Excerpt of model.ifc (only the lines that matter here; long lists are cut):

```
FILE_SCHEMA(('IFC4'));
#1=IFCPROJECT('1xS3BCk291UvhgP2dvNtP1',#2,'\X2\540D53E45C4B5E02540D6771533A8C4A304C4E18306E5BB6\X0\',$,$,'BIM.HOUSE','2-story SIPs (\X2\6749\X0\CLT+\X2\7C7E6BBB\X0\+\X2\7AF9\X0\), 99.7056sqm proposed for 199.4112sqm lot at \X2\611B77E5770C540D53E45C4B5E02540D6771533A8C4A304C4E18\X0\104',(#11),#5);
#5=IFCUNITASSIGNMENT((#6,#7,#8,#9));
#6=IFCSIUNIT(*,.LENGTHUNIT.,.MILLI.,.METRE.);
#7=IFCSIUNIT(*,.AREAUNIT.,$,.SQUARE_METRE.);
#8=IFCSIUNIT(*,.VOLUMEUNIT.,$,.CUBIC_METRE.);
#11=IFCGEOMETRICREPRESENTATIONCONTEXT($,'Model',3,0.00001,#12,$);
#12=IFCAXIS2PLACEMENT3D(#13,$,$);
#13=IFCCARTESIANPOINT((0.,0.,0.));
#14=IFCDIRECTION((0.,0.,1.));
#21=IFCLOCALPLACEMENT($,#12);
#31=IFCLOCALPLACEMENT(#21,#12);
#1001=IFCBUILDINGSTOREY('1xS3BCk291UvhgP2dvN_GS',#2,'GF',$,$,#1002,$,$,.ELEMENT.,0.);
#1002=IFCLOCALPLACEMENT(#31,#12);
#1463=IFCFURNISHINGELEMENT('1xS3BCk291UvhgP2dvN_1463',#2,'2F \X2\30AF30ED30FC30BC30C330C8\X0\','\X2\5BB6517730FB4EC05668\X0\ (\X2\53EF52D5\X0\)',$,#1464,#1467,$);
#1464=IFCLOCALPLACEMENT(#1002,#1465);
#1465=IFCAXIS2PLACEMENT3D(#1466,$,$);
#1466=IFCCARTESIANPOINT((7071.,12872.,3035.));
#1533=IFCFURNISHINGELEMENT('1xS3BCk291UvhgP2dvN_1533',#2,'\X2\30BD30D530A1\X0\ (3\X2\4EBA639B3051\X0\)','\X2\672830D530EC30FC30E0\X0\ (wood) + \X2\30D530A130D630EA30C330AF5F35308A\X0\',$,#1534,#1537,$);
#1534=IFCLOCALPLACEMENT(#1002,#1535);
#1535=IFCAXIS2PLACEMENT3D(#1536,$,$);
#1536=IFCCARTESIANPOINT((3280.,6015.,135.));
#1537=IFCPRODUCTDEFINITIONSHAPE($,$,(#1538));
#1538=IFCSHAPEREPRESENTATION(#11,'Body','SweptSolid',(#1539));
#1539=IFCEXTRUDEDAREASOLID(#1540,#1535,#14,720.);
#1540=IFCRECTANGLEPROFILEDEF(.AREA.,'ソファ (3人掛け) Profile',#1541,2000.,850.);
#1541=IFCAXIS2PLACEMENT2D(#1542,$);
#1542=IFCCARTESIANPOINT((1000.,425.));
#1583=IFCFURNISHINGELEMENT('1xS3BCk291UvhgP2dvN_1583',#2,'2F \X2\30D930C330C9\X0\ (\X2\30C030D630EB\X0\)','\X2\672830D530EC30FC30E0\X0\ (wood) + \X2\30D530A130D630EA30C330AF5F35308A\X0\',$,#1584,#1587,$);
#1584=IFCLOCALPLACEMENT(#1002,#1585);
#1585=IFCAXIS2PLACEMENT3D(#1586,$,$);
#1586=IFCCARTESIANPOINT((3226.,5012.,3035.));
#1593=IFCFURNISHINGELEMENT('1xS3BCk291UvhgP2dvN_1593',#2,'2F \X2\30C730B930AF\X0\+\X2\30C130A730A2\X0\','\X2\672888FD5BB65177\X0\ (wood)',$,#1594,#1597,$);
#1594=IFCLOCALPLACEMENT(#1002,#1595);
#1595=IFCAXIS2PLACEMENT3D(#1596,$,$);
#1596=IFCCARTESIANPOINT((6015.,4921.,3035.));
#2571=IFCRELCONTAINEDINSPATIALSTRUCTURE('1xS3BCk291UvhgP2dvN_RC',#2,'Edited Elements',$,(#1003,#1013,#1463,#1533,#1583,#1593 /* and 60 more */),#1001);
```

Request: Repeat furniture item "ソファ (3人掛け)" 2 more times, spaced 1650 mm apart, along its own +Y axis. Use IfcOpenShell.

```python
import ifcopenshell
import ifcopenshell.api.geometry
import ifcopenshell.api.root
import ifcopenshell.util.element
import ifcopenshell.util.placement
import ifcopenshell.util.unit

model = ifcopenshell.open("model.ifc")
unit_scale = ifcopenshell.util.unit.calculate_unit_scale(model)


def reuse_history(source, copy):
    """copy_class also copies each property set's owner history, people and application; keep the originals."""
    for rel in copy.IsDefinedBy:
        if rel.is_a("IfcRelDefinesByProperties") and (history := rel.RelatingPropertyDefinition.OwnerHistory):
            rel.RelatingPropertyDefinition.OwnerHistory = source.OwnerHistory
            ifcopenshell.util.element.remove_deep2(model, history)


source = model.by_guid("1xS3BCk291UvhgP2dvN_1533")
base = ifcopenshell.util.placement.get_local_placement(source.ObjectPlacement)
step = base[:3, 1] * 1.65 / unit_scale

for i in range(1, 3):
    copy = ifcopenshell.api.root.copy_class(model, product=source)
    copy.Representation = ifcopenshell.util.element.copy_deep(
        model, source.Representation, exclude=["IfcGeometricRepresentationContext", "IfcRepresentationMap"]
    )
    reuse_history(source, copy)
    matrix = base.copy()
    matrix[:3, 3] += i * step
    print("added at", matrix[:3, 3].round(3) + 0.0)
    ifcopenshell.api.geometry.edit_object_placement(model, product=copy, matrix=matrix, is_si=False)

model.write("model_rev.ifc")
```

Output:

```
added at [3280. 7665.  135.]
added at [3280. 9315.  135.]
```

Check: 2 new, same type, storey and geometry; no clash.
